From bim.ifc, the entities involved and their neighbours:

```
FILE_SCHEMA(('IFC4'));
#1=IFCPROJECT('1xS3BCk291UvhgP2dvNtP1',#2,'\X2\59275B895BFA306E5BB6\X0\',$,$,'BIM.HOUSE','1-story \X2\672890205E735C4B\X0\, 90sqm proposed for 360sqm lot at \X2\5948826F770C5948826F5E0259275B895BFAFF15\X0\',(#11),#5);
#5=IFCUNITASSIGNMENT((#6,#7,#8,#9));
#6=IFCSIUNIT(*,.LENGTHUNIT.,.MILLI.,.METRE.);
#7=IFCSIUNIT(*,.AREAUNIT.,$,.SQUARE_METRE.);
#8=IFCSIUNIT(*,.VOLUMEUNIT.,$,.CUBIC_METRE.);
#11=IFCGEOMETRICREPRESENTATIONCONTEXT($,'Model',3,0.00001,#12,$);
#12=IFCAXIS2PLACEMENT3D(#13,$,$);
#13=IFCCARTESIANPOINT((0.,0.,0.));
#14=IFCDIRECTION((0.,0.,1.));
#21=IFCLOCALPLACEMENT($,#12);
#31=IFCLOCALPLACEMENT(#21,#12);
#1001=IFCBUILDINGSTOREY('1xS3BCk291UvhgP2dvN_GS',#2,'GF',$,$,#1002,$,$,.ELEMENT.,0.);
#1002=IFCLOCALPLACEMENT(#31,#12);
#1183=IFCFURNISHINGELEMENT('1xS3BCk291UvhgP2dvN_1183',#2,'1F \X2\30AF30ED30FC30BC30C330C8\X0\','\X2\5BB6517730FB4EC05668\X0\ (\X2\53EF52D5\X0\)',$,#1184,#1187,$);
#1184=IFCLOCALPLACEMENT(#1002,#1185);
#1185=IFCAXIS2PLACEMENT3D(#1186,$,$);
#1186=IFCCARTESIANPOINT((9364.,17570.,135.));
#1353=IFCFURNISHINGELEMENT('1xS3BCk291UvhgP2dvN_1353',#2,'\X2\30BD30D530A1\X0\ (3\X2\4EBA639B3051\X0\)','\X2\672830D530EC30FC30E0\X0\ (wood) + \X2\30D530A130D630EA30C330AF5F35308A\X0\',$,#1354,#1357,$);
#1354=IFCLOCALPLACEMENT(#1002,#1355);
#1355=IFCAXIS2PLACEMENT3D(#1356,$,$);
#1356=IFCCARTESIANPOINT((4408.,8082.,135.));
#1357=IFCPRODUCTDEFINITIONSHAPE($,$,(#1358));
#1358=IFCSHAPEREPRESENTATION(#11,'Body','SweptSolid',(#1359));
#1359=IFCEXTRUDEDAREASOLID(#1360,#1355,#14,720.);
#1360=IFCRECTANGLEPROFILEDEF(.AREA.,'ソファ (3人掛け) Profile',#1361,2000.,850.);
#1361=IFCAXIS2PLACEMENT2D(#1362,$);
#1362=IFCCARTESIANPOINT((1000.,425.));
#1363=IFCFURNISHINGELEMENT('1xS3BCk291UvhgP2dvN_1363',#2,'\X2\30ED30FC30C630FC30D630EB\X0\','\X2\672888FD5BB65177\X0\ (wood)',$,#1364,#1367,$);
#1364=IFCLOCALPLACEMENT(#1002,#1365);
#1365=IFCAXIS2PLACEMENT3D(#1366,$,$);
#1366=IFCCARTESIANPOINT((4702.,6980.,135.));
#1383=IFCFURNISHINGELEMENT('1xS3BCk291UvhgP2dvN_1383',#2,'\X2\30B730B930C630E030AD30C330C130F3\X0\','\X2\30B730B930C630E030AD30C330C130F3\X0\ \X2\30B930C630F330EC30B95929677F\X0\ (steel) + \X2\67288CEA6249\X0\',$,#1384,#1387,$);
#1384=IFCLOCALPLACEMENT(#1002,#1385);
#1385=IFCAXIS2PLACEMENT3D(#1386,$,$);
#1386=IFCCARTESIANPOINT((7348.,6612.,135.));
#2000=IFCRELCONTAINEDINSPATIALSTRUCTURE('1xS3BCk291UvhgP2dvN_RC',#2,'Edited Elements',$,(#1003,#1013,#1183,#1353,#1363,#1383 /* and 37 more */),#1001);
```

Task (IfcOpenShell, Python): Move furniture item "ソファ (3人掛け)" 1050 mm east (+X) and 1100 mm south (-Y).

```python
import ifcopenshell
import ifcopenshell.api.geometry
import ifcopenshell.util.placement

model = ifcopenshell.open("bim.ifc")

item = model.by_guid("1xS3BCk291UvhgP2dvN_1353")
matrix = ifcopenshell.util.placement.get_local_placement(item.ObjectPlacement)
matrix[0, 3] += 1050.0
matrix[1, 3] -= 1100.0
ifcopenshell.api.geometry.edit_object_placement(model, product=item, matrix=matrix, is_si=False)

print(ifcopenshell.util.placement.get_local_placement(item.ObjectPlacement).round(3) + 0.0)

model.write("bim-out.ifc")
```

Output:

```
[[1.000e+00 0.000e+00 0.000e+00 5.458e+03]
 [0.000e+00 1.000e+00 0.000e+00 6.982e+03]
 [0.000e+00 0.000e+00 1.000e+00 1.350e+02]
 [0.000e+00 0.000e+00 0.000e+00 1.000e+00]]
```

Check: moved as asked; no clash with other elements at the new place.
